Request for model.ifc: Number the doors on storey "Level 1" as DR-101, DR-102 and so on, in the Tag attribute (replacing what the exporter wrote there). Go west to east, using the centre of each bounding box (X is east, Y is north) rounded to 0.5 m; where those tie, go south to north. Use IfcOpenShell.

First a look at what the model holds.

```python
import ifcopenshell
import ifcopenshell.util.element
import ifcopenshell.util.placement

model = ifcopenshell.open("model.ifc")
print(model.schema)
storey = next(s for s in model.by_type("IfcBuildingStorey") if s.Name == "Level 1")
doors = [e for e in ifcopenshell.util.element.get_decomposition(storey) if e.is_a("IfcDoor")]
for e in sorted(doors, key=lambda e: e.id()):
    origin = ifcopenshell.util.placement.get_local_placement(e.ObjectPlacement)[:3, 3]
    print(e.id(), e.Tag, e.Name, origin.round(2) + 0.0, sep=" | ")
```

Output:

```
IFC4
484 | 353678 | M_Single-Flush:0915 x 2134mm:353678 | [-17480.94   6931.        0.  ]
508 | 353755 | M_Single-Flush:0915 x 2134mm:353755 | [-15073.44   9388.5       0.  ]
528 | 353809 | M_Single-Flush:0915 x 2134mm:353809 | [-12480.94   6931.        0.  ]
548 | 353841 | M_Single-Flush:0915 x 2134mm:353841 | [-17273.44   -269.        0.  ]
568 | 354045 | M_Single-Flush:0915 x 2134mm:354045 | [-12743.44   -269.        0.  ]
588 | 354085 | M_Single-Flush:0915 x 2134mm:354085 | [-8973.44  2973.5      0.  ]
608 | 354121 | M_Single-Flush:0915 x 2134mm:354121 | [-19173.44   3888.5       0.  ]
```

```python
import ifcopenshell
import ifcopenshell.geom
import ifcopenshell.util.element
import ifcopenshell.util.shape

model = ifcopenshell.open("model.ifc")
settings = ifcopenshell.geom.settings()
settings.set("use-world-coords", True)


def centre(element):
    shape = ifcopenshell.geom.create_shape(settings, element)
    return ifcopenshell.util.shape.get_bbox_centroid(shape.geometry)


storey = next(s for s in model.by_type("IfcBuildingStorey") if s.Name == "Level 1")
doors = [e for e in ifcopenshell.util.element.get_decomposition(storey) if e.is_a("IfcDoor")]

# Insertion points can sit at a corner or the storey origin, so sort by the geometry (in metres).
centres = {e: centre(e) for e in doors}
doors.sort(key=lambda e: (round(centres[e][0] / 0.5), centres[e][1]))

for i, e in enumerate(doors, start=1):
    number = f"DR-1{i:02d}"
    e.Tag = number
    print(e.id(), number)

model.write("model_v2.ifc")
```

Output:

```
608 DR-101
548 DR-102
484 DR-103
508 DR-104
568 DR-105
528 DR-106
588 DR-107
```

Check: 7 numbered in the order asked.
